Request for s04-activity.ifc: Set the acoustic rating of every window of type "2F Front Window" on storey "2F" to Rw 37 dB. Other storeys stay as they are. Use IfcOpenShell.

First a look at what the model holds.

```python
import ifcopenshell
import ifcopenshell.util.element

model = ifcopenshell.open("s04-activity.ifc")
print(model.schema)
storey = next(s for s in model.by_type("IfcBuildingStorey") if s.Name == "2F")
windows = [e for e in ifcopenshell.util.element.get_decomposition(storey) if e.is_a("IfcWindow")]
seen = {}
for e in windows:
    element_type = ifcopenshell.util.element.get_type(e)
    key = (element_type.Name if element_type != e and element_type else None, ifcopenshell.util.element.get_pset(e, "Pset_WindowCommon", "AcousticRating"))
    seen[key] = seen.get(key, 0) + 1
for (name, value), count in sorted(seen.items(), key=str):
    print(count, "x", name, "|", value)
```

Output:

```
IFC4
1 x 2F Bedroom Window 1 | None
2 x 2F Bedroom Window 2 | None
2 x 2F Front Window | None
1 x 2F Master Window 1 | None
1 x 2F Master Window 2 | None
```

```python
import ifcopenshell
import ifcopenshell.api.pset
import ifcopenshell.util.element

model = ifcopenshell.open("s04-activity.ifc")

storey = next(s for s in model.by_type("IfcBuildingStorey") if s.Name == "2F")
windows = [e for e in ifcopenshell.util.element.get_decomposition(storey) if e.is_a("IfcWindow")]

count = 0
for e in windows:
    element_type = ifcopenshell.util.element.get_type(e)
    if element_type in (None, e) or element_type.Name != "2F Front Window":
        continue
    # add_pset returns the element's existing set when there is one.
    pset = ifcopenshell.api.pset.add_pset(model, product=e, name="Pset_WindowCommon")
    ifcopenshell.api.pset.edit_pset(model, pset=pset, properties={"AcousticRating": "Rw 37 dB"})
    count += 1

print(count, "windows updated")

model.write("s04-activity_edited.ifc")
```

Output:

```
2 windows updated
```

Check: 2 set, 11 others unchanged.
